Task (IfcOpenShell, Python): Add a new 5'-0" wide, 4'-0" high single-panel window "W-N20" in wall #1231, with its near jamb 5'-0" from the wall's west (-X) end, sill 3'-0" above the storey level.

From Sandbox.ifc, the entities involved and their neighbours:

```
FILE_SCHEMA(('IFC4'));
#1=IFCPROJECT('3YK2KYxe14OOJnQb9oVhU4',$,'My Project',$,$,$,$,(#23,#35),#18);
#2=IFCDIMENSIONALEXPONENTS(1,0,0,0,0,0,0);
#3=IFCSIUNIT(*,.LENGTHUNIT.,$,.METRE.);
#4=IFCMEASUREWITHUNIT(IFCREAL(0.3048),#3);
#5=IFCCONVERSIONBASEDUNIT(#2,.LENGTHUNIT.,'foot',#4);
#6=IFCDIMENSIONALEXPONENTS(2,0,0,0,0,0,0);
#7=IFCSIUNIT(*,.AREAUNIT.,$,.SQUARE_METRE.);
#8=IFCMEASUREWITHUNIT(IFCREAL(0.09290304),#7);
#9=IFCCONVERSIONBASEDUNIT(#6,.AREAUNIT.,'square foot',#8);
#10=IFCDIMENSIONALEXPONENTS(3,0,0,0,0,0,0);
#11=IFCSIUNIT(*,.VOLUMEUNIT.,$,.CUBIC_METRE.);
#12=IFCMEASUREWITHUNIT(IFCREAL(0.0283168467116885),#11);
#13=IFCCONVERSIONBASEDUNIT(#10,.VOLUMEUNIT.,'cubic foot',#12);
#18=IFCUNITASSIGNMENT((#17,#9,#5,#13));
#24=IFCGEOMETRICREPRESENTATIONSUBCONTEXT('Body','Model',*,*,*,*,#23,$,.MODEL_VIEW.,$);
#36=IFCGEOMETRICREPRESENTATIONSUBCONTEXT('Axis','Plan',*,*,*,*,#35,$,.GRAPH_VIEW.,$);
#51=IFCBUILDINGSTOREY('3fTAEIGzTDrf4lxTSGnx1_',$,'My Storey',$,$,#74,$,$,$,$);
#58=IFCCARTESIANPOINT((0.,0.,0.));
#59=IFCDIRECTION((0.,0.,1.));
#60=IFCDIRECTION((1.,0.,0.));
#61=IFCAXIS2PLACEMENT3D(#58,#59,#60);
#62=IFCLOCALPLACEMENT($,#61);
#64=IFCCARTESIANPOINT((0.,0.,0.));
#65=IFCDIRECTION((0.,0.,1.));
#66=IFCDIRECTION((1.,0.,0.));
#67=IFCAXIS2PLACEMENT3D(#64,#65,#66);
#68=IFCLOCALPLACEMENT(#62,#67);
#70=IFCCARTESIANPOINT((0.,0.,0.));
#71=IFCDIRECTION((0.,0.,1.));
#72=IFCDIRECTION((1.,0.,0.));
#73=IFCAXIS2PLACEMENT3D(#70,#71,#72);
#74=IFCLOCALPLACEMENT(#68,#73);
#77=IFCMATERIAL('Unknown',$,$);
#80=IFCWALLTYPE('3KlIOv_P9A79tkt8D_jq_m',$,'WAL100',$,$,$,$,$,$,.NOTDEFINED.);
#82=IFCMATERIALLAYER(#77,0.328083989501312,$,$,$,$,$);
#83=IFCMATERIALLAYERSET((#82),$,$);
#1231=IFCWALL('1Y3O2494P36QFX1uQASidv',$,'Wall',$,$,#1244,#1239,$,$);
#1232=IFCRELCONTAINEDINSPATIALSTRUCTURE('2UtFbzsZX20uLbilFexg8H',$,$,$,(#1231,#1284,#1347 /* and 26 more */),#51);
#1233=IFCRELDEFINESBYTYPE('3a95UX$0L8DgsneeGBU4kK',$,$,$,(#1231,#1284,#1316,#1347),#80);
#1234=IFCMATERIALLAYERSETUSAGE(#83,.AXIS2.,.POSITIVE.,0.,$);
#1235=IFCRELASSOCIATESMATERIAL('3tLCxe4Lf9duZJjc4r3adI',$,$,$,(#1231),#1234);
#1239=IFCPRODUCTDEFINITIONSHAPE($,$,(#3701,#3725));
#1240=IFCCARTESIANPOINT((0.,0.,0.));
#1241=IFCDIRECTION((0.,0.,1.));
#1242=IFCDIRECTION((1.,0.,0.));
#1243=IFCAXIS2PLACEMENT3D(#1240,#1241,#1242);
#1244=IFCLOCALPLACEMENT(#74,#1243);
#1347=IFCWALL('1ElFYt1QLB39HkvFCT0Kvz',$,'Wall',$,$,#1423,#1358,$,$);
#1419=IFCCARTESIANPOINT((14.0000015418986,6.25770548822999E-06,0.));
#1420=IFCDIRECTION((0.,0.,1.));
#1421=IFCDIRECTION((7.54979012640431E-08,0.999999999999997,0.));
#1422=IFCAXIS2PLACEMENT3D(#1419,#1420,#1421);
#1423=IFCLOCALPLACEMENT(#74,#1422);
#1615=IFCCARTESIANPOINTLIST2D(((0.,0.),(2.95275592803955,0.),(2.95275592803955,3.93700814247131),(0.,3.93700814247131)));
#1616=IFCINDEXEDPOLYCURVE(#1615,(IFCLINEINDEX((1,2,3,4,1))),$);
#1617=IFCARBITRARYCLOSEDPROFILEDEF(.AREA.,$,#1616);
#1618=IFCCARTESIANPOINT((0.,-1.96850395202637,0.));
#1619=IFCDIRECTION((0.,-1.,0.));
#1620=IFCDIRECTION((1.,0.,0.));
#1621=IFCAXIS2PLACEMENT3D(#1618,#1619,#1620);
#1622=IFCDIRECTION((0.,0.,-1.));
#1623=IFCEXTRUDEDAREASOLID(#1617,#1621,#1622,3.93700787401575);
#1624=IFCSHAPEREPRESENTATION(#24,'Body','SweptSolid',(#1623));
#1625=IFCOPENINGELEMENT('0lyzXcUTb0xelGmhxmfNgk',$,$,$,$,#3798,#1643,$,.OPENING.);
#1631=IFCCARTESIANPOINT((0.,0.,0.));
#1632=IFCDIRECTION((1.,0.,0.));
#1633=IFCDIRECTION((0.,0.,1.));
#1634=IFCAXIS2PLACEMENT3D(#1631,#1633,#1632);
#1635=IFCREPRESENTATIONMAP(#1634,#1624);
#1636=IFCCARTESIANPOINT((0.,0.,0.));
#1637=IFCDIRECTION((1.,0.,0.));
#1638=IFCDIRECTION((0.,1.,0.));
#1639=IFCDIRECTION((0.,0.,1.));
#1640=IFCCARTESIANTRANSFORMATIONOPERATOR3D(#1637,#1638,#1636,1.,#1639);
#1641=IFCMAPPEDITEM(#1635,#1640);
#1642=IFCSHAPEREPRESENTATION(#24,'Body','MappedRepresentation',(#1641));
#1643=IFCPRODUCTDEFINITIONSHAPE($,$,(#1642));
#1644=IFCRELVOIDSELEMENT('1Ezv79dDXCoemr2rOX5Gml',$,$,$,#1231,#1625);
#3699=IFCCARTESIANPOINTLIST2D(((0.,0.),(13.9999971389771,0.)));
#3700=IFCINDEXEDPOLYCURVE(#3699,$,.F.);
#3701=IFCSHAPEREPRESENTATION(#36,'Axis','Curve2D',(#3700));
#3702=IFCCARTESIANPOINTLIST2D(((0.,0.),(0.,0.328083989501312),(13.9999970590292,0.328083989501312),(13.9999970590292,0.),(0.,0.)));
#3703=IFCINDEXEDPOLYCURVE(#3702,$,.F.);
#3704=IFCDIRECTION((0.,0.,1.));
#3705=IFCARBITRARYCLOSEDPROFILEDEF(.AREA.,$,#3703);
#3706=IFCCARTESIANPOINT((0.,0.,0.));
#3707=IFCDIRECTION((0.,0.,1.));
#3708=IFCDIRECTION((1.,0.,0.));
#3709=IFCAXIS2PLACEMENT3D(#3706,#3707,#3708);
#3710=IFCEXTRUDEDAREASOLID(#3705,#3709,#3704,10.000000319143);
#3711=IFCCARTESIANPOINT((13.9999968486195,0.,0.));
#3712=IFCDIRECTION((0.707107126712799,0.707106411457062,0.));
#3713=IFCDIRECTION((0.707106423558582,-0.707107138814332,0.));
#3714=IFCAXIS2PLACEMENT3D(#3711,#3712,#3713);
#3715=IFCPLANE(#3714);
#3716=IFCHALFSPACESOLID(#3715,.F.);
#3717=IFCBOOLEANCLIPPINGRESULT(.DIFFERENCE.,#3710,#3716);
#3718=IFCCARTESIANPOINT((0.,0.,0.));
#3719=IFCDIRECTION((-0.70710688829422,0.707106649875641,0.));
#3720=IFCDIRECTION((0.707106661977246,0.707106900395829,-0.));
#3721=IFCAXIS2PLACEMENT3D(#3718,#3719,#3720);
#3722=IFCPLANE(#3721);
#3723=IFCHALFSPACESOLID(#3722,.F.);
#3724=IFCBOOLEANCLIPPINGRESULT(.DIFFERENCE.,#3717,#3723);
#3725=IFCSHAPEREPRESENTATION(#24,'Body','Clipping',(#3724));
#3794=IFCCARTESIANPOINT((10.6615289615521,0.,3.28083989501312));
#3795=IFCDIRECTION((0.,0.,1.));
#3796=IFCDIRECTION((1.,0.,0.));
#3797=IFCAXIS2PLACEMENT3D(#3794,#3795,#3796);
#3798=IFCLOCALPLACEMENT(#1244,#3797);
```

```python
import numpy as np
import ifcopenshell
import ifcopenshell.api.feature
import ifcopenshell.api.geometry
import ifcopenshell.api.root
import ifcopenshell.api.spatial
import ifcopenshell.geom
import ifcopenshell.util.element
import ifcopenshell.util.placement
import ifcopenshell.util.representation
import ifcopenshell.util.shape
import ifcopenshell.util.unit

model = ifcopenshell.open("Sandbox.ifc")
unit_scale = ifcopenshell.util.unit.calculate_unit_scale(model)
settings = ifcopenshell.geom.settings()


def volume(element):
    """Net volume in cubic metres, openings subtracted."""
    shape = ifcopenshell.geom.create_shape(settings, element)
    return ifcopenshell.util.shape.get_volume(shape.geometry)


wall = model.by_guid("1Y3O2494P36QFX1uQASidv")
storey = ifcopenshell.util.element.get_container(wall, ifc_class="IfcBuildingStorey")
context = ifcopenshell.util.representation.get_context(model, "Model", "Body", "MODEL_VIEW")
before = volume(wall)

width, height, from_end, sill = 1.524, 1.2192, 1.524, 0.9144  # metres

# The wall runs along its own X axis, and the end named is its -X end.
wall_shape = ifcopenshell.geom.create_shape(settings, wall)
x, y, z = ifcopenshell.util.shape.get_vertices(wall_shape.geometry).T
start = x.min() + from_end
face, thickness = float(y.min()), float(y.max() - y.min())
wall_matrix = ifcopenshell.util.placement.get_local_placement(wall.ObjectPlacement)
level = ifcopenshell.util.placement.get_local_placement(storey.ObjectPlacement)[2, 3]


def in_wall(x, y):
    """Placement at x, y metres in the wall's axes, at sill height."""
    matrix = wall_matrix.copy()
    matrix[:, 3] = wall_matrix @ np.array([x / unit_scale, y / unit_scale, 0.0, 1.0])
    matrix[2, 3] = level + sill / unit_scale
    return matrix


# Opening: a box that overshoots both wall faces by 50 mm.
opening = ifcopenshell.api.root.create_entity(model, ifc_class="IfcOpeningElement", predefined_type="OPENING")
box = ifcopenshell.api.geometry.add_wall_representation(
    model, context=context, length=width, height=height, thickness=thickness + 0.1
)
ifcopenshell.api.geometry.assign_representation(model, product=opening, representation=box)
ifcopenshell.api.geometry.edit_object_placement(model, product=opening, matrix=in_wall(start, face - 0.05), is_si=False)
ifcopenshell.api.feature.add_feature(model, feature=opening, element=wall)

window = ifcopenshell.api.root.create_entity(model, ifc_class="IfcWindow", name="W-N20", predefined_type="WINDOW")
window.OverallWidth, window.OverallHeight = width / unit_scale, height / unit_scale
window.PartitioningType = "SINGLE_PANEL"
body = ifcopenshell.api.geometry.add_window_representation(
    model,
    context=context,
    overall_width=window.OverallWidth,
    overall_height=window.OverallHeight,
    partition_type="SINGLE_PANEL",
)
ifcopenshell.api.geometry.assign_representation(model, product=window, representation=body)
ifcopenshell.api.spatial.assign_container(model, products=[window], relating_structure=storey)
ifcopenshell.api.feature.add_filling(model, opening=opening, element=window)

# Centre the window in the wall's thickness.
ifcopenshell.api.geometry.edit_object_placement(model, product=window, matrix=in_wall(start, face), is_si=False)
window_shape = ifcopenshell.geom.create_shape(settings, window)
depth = ifcopenshell.util.shape.get_vertices(window_shape.geometry)[:, 1]
offset = face + thickness / 2 - (depth.min() + depth.max()) / 2
ifcopenshell.api.geometry.edit_object_placement(model, product=window, matrix=in_wall(start, offset), is_si=False)

after = volume(wall)

print(f"wall volume {before:.3f} -> {after:.3f} m3")

model.write("Sandbox_edited.ifc")
```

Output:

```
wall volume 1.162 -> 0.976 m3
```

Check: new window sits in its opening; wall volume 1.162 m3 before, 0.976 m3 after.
